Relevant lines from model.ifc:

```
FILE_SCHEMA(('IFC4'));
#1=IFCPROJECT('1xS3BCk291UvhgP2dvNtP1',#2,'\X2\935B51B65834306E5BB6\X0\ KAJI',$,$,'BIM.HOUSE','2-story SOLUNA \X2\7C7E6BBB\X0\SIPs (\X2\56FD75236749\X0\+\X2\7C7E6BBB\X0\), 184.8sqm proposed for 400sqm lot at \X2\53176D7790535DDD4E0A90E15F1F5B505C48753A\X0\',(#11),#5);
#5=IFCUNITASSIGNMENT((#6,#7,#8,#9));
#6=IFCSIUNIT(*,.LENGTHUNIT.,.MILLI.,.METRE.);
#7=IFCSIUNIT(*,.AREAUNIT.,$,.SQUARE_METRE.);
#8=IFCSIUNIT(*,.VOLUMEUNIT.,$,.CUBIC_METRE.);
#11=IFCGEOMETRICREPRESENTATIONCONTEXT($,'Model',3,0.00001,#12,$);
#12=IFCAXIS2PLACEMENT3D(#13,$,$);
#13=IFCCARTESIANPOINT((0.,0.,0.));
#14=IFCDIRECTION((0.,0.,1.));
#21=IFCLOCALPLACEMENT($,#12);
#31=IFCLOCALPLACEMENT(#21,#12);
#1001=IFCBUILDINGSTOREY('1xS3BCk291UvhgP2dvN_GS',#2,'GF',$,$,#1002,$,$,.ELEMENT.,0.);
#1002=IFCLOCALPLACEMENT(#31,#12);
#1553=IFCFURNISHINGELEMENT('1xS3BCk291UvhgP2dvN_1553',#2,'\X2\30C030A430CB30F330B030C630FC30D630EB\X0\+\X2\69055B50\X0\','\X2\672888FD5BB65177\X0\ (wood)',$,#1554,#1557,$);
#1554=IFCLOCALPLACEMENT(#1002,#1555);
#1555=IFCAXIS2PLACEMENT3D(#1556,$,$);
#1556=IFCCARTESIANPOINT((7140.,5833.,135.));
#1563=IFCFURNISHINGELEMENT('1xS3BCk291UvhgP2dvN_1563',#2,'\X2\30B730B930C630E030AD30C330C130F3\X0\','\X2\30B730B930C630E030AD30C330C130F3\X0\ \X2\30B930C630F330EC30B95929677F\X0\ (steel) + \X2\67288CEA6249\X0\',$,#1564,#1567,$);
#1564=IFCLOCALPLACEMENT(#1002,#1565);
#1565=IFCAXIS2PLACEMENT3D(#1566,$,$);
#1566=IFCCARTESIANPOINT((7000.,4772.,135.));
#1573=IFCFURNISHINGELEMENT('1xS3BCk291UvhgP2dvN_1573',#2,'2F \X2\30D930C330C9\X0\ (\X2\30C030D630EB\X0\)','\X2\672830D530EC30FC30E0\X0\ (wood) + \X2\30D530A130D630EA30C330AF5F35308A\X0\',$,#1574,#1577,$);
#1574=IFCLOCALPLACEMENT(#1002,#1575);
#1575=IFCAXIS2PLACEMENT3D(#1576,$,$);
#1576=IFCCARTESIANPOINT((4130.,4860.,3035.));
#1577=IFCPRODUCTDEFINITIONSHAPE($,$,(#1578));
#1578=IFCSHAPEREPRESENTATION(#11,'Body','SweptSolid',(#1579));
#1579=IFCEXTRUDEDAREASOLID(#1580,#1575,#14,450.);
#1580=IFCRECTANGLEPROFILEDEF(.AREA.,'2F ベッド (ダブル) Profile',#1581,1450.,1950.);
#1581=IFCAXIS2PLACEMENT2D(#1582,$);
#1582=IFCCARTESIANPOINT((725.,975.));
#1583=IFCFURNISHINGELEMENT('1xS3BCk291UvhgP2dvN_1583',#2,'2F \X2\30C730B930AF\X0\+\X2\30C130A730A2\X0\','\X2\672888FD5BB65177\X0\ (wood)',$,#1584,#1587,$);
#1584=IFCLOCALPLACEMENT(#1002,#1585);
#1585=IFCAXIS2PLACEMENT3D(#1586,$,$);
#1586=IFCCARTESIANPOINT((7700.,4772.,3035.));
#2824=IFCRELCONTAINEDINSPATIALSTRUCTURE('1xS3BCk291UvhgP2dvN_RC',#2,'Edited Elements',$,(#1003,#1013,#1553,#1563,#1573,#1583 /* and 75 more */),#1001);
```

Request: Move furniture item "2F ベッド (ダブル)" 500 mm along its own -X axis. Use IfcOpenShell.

```python
import ifcopenshell
import ifcopenshell.api.geometry
import ifcopenshell.util.placement
import ifcopenshell.util.unit

model = ifcopenshell.open("model.ifc")
unit_scale = ifcopenshell.util.unit.calculate_unit_scale(model)

item = model.by_id(1573)
matrix = ifcopenshell.util.placement.get_local_placement(item.ObjectPlacement)
matrix[:3, 3] -= matrix[:3, 0] * 0.5 / unit_scale
ifcopenshell.api.geometry.edit_object_placement(model, product=item, matrix=matrix, is_si=False)

print(ifcopenshell.util.placement.get_local_placement(item.ObjectPlacement).round(3) + 0.0)

model.write("model_updated.ifc")
```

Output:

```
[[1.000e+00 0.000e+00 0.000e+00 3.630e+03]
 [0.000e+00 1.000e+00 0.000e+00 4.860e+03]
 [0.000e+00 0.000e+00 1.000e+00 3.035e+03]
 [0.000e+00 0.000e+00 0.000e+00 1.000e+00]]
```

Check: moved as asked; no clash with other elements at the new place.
